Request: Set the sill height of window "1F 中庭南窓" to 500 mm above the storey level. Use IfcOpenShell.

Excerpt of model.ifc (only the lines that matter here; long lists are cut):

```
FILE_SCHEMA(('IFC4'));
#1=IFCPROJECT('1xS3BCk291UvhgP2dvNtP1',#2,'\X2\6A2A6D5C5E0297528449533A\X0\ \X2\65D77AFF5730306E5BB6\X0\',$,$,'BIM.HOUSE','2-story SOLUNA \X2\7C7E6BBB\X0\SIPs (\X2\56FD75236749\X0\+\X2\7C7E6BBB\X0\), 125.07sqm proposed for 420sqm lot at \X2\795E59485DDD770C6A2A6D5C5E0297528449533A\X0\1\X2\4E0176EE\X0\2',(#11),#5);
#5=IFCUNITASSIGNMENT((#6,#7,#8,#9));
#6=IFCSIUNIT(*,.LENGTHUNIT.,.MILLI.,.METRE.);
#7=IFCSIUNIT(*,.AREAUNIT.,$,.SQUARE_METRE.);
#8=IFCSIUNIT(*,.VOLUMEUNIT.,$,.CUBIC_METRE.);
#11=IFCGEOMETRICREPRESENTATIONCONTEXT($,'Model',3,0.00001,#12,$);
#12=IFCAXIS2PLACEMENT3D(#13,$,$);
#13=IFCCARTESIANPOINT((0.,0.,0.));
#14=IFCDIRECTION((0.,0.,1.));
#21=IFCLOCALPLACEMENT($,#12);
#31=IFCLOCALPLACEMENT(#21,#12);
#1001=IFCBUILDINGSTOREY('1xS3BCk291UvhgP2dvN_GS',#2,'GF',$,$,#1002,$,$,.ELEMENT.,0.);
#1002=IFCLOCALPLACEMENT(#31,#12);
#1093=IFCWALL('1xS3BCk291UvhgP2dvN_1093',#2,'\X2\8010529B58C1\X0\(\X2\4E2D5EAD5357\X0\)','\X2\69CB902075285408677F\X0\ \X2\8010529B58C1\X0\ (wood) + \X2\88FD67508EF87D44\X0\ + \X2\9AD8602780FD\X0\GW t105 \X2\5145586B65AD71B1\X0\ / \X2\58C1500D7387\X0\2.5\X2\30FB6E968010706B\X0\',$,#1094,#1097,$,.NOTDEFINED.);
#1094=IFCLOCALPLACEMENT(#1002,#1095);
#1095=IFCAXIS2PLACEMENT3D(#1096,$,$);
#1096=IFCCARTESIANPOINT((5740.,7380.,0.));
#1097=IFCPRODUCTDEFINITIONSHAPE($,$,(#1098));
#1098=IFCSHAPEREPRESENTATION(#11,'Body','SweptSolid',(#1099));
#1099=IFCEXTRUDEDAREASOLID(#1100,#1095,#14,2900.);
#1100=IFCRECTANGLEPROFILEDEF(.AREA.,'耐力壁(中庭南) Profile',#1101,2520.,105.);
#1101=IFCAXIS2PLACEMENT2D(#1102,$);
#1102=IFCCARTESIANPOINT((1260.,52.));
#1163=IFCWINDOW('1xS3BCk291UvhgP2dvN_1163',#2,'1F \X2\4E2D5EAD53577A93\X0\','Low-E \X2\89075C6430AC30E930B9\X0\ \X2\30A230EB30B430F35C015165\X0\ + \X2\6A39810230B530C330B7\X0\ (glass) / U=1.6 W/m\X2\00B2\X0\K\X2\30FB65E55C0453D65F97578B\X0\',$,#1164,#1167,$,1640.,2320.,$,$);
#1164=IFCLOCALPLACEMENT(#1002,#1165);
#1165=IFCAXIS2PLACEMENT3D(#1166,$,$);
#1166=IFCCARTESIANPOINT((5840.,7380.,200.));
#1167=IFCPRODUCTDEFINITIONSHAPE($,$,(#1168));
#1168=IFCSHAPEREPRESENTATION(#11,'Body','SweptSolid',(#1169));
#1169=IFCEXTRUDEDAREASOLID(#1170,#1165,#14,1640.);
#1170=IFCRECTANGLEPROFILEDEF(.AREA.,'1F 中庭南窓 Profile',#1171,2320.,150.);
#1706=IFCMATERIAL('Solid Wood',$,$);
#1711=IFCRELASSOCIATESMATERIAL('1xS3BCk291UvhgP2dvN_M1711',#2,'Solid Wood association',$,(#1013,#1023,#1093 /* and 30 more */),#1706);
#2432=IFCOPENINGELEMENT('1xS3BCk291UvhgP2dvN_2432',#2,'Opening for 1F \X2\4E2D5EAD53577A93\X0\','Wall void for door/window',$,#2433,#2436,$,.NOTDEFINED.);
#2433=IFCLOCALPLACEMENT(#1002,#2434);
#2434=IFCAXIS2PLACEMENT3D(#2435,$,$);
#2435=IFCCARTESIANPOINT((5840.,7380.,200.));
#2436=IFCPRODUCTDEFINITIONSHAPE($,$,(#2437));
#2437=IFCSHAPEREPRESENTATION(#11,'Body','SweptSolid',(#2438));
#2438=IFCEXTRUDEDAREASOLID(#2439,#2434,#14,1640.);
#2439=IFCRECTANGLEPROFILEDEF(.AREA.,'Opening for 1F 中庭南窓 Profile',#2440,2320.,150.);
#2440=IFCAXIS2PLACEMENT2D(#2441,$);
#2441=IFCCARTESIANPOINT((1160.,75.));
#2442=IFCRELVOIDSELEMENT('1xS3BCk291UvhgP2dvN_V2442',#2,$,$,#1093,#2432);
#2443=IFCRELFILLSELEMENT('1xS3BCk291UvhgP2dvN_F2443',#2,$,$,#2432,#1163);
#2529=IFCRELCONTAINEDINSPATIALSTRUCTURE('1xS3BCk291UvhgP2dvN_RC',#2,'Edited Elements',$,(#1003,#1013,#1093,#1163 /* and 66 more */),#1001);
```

```python
import numpy as np
import ifcopenshell
import ifcopenshell.api.geometry
import ifcopenshell.geom
import ifcopenshell.util.element
import ifcopenshell.util.placement
import ifcopenshell.util.shape
import ifcopenshell.util.unit

model = ifcopenshell.open("model.ifc")
unit_scale = ifcopenshell.util.unit.calculate_unit_scale(model)

window = model.by_guid("1xS3BCk291UvhgP2dvN_1163")
opening = window.FillsVoids[0].RelatingOpeningElement
storey = ifcopenshell.util.element.get_container(window, ifc_class="IfcBuildingStorey")
level = ifcopenshell.util.placement.get_local_placement(storey.ObjectPlacement)[2, 3]

# The opening's origin need not be at the sill, so measure its lowest point.
shape = ifcopenshell.geom.create_shape(ifcopenshell.geom.settings(), opening)
bottom = ifcopenshell.util.shape.get_shape_bottom_elevation(shape, shape.geometry) / unit_scale
dz = level + 0.5 / unit_scale - bottom

shift = np.array([0.0, 0.0, dz])
# The window is not placed relative to its opening, so move both.
for product in (opening, window):
    matrix = ifcopenshell.util.placement.get_local_placement(product.ObjectPlacement)
    matrix[:3, 3] += shift
    ifcopenshell.api.geometry.edit_object_placement(model, product=product, matrix=matrix, is_si=False)

print(f"moved by {dz * unit_scale:+.3f} m")

model.write("model_updated.ifc")
```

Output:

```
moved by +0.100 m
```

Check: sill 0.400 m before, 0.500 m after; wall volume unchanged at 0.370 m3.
